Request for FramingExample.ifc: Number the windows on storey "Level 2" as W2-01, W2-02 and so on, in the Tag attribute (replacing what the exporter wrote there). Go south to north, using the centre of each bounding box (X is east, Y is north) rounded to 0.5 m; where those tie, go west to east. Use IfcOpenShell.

First a look at what the model holds.

```python
import ifcopenshell
import ifcopenshell.util.element
import ifcopenshell.util.placement

model = ifcopenshell.open("FramingExample.ifc")
print(model.schema)
storey = next(s for s in model.by_type("IfcBuildingStorey") if s.Name == "Level 2")
windows = [e for e in ifcopenshell.util.element.get_decomposition(storey) if e.is_a("IfcWindow")]
for e in sorted(windows, key=lambda e: e.id()):
    origin = ifcopenshell.util.placement.get_local_placement(e.ObjectPlacement)[:3, 3]
    print(e.id(), e.Tag, e.Name, origin.round(2) + 0.0, sep=" | ")
```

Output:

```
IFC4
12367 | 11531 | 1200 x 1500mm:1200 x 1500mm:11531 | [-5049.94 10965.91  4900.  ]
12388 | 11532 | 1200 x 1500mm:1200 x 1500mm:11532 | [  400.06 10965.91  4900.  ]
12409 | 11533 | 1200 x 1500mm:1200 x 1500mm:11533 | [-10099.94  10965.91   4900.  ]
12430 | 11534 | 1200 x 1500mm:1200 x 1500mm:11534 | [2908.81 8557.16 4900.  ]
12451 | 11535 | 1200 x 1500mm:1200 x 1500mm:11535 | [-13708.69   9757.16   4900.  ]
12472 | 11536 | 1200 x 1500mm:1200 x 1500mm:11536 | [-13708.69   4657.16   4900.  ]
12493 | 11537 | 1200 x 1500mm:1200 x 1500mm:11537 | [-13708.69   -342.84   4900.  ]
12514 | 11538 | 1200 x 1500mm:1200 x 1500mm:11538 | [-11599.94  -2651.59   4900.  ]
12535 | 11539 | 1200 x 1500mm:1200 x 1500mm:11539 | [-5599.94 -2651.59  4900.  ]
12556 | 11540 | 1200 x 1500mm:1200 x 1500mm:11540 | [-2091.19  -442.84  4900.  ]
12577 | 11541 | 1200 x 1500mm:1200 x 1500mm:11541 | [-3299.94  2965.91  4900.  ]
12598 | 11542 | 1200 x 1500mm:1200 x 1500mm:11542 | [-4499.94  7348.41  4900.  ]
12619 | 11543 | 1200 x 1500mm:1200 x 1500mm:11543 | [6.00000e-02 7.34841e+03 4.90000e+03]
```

```python
import ifcopenshell
import ifcopenshell.geom
import ifcopenshell.util.element
import ifcopenshell.util.shape

model = ifcopenshell.open("FramingExample.ifc")
settings = ifcopenshell.geom.settings()
settings.set("use-world-coords", True)


def centre(element):
    shape = ifcopenshell.geom.create_shape(settings, element)
    return ifcopenshell.util.shape.get_bbox_centroid(shape.geometry)


storey = next(s for s in model.by_type("IfcBuildingStorey") if s.Name == "Level 2")
windows = [e for e in ifcopenshell.util.element.get_decomposition(storey) if e.is_a("IfcWindow")]

# Insertion points can sit at a corner or the storey origin, so sort by the geometry (in metres).
centres = {e: centre(e) for e in windows}
windows.sort(key=lambda e: (round(centres[e][1] / 0.5), centres[e][0]))

for i, e in enumerate(windows, start=1):
    number = f"W2-{i:02d}"
    e.Tag = number
    print(e.id(), number)

model.write("FramingExample_rev.ifc")
```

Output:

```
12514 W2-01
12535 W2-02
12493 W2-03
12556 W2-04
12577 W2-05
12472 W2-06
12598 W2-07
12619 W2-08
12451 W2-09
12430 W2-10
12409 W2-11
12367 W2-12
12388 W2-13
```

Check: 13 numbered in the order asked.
